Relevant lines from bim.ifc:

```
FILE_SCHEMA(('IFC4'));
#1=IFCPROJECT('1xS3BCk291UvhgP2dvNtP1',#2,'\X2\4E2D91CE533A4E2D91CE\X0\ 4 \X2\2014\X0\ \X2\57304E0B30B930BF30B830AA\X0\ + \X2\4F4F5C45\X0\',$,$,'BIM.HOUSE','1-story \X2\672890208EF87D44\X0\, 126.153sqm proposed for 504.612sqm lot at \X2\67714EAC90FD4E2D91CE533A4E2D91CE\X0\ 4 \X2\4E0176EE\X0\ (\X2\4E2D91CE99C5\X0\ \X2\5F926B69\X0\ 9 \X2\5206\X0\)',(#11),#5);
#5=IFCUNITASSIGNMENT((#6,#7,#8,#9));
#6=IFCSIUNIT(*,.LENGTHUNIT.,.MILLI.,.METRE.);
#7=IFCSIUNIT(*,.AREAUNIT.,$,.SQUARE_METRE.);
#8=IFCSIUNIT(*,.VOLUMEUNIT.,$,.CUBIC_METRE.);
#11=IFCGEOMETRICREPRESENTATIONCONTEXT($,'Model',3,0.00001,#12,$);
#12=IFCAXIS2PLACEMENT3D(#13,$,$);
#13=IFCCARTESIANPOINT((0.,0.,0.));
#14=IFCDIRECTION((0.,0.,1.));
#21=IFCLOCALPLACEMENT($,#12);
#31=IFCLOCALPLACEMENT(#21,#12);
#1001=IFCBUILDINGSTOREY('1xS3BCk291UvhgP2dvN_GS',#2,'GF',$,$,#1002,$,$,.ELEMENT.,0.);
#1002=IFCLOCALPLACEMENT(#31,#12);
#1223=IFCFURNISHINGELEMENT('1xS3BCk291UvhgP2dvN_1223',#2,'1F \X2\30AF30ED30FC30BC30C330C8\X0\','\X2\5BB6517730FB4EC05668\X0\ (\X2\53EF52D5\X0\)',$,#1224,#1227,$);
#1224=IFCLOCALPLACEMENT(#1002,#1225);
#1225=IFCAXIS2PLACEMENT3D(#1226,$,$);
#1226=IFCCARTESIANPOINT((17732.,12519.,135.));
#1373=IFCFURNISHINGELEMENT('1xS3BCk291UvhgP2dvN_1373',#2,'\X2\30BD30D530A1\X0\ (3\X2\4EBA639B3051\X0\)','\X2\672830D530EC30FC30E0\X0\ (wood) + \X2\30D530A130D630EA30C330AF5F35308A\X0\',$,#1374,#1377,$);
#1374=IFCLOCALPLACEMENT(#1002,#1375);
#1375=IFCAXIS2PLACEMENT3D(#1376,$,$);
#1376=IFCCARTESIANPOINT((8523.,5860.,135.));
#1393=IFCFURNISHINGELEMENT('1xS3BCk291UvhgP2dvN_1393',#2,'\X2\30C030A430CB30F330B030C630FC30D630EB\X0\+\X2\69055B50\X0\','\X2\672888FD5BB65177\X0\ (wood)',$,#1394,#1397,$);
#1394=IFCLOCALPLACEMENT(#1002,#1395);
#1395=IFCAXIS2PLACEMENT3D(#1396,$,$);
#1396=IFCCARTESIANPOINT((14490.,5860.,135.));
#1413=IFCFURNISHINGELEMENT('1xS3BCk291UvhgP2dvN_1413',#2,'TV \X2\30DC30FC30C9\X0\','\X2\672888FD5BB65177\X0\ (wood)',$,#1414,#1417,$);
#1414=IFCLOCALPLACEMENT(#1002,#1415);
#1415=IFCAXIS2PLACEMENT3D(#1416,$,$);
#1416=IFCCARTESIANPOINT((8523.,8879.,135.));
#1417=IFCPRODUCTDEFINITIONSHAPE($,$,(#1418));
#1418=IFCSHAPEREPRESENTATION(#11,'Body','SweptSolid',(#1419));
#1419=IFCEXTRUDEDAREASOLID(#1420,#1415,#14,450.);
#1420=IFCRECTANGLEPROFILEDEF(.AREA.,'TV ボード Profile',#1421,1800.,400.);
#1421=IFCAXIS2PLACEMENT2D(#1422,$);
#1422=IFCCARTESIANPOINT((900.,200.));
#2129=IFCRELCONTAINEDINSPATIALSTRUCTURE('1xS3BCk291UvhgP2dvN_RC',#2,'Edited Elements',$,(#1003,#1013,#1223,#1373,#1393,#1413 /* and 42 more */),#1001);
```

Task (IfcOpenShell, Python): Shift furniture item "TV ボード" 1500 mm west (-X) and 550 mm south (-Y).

```python
import ifcopenshell
import ifcopenshell.api.geometry
import ifcopenshell.util.placement

model = ifcopenshell.open("bim.ifc")

item = model.by_id(1413)
matrix = ifcopenshell.util.placement.get_local_placement(item.ObjectPlacement)
matrix[0, 3] -= 1500.0
matrix[1, 3] -= 550.0
ifcopenshell.api.geometry.edit_object_placement(model, product=item, matrix=matrix, is_si=False)

print(ifcopenshell.util.placement.get_local_placement(item.ObjectPlacement).round(3) + 0.0)

model.write("bim-out.ifc")
```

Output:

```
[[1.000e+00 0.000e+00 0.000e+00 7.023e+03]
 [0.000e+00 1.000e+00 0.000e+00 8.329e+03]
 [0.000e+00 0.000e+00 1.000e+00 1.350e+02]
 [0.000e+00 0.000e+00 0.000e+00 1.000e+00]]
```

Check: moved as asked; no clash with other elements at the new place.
